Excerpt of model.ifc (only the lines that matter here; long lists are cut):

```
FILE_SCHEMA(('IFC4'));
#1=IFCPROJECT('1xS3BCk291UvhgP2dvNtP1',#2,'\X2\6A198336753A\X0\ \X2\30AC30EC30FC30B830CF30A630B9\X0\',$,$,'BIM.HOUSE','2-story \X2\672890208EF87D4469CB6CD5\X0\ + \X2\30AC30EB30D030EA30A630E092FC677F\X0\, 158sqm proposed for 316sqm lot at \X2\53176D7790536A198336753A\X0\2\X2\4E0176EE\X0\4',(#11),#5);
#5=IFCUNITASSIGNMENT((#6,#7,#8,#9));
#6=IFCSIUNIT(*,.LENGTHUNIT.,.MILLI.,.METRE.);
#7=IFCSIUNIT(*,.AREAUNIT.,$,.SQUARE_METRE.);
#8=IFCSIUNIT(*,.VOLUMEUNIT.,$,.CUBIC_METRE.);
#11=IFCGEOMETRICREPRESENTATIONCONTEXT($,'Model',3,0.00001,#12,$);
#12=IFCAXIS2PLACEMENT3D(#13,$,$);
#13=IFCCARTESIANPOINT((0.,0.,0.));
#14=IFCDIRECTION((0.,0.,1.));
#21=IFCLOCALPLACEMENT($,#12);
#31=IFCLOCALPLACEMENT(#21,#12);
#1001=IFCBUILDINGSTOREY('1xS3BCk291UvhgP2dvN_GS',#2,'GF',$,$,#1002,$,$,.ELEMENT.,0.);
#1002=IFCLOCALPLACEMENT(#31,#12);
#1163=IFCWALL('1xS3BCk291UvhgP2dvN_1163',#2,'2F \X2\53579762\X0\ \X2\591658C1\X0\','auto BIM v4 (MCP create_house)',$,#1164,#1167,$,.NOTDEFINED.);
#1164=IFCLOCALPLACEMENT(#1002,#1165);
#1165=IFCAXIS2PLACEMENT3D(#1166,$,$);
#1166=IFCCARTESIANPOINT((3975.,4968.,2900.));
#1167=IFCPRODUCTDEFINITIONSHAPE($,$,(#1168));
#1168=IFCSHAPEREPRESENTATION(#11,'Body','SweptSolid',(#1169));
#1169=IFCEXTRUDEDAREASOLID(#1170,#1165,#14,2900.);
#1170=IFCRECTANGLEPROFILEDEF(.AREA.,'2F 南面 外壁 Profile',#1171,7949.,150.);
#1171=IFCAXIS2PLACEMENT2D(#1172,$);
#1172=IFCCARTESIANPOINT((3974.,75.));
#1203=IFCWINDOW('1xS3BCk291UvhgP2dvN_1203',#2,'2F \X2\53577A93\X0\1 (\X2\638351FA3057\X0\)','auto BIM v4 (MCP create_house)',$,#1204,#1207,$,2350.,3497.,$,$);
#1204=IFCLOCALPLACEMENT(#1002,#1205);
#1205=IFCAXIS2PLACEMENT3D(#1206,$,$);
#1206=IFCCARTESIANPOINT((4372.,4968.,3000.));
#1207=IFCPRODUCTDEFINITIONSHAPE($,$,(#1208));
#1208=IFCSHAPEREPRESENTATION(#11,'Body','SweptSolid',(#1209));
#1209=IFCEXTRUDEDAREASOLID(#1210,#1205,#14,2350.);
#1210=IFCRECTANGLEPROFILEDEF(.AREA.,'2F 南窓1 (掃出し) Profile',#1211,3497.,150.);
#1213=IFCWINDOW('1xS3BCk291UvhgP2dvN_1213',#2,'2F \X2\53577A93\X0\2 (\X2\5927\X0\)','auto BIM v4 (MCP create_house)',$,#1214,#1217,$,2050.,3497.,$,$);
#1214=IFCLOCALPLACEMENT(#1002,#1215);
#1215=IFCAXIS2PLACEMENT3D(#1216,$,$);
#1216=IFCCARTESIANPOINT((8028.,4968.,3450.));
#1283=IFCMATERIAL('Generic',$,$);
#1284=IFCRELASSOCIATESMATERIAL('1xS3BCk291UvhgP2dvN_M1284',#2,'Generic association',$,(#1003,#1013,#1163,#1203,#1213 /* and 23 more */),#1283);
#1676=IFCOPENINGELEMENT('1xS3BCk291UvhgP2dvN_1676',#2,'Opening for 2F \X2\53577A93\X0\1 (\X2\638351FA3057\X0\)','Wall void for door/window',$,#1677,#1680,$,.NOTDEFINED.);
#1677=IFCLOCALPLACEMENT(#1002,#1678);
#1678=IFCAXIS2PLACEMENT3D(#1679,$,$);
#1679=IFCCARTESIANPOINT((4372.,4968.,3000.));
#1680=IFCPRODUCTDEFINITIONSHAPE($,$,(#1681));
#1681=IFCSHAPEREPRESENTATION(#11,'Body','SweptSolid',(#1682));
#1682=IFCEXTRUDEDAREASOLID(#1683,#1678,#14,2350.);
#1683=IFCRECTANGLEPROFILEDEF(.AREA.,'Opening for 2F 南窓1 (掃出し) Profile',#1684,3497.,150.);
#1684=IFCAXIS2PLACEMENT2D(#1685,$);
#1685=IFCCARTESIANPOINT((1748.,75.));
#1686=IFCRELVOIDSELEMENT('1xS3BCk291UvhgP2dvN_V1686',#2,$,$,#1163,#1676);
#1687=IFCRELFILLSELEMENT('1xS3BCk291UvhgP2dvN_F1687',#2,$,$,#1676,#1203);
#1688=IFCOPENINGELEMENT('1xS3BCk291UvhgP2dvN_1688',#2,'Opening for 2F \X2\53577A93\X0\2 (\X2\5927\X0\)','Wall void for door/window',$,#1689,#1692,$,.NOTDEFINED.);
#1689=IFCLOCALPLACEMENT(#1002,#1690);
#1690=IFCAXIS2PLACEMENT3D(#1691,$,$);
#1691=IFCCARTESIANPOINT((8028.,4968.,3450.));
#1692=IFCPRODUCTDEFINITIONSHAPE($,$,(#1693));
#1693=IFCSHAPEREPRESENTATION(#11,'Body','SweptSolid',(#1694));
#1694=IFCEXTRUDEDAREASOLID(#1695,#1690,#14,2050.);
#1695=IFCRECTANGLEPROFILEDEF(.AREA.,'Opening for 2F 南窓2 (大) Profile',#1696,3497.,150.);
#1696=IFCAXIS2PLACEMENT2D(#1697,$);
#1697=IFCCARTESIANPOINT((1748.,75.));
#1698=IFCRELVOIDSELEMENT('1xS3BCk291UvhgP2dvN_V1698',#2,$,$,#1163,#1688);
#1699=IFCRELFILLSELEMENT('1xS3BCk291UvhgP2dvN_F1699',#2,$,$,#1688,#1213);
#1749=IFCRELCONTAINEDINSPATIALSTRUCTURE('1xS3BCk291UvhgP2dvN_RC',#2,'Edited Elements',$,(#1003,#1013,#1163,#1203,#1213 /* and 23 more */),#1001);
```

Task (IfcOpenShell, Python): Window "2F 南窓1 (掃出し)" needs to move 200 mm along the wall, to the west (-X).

```python
import ifcopenshell
import ifcopenshell.api.geometry
import ifcopenshell.util.placement

model = ifcopenshell.open("model.ifc")

window = model.by_guid("1xS3BCk291UvhgP2dvN_1203")
opening = window.FillsVoids[0].RelatingOpeningElement
wall = opening.VoidsElements[0].RelatingBuildingElement

wall_matrix = ifcopenshell.util.placement.get_local_placement(wall.ObjectPlacement)
shift = wall_matrix[:3, 0] * -200.0
before = ifcopenshell.util.placement.get_local_placement(window.ObjectPlacement)[:3, 3].copy()

# The window is not placed relative to its opening, so move both.
for product in (opening, window):
    matrix = ifcopenshell.util.placement.get_local_placement(product.ObjectPlacement)
    matrix[:3, 3] += shift
    ifcopenshell.api.geometry.edit_object_placement(model, product=product, matrix=matrix, is_si=False)

after = ifcopenshell.util.placement.get_local_placement(window.ObjectPlacement)[:3, 3]
print("window moved by", (after - before).round(3) + 0.0)

model.write("model_v2.ifc")
```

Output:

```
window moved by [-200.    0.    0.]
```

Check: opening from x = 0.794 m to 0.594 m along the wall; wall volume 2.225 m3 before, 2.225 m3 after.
